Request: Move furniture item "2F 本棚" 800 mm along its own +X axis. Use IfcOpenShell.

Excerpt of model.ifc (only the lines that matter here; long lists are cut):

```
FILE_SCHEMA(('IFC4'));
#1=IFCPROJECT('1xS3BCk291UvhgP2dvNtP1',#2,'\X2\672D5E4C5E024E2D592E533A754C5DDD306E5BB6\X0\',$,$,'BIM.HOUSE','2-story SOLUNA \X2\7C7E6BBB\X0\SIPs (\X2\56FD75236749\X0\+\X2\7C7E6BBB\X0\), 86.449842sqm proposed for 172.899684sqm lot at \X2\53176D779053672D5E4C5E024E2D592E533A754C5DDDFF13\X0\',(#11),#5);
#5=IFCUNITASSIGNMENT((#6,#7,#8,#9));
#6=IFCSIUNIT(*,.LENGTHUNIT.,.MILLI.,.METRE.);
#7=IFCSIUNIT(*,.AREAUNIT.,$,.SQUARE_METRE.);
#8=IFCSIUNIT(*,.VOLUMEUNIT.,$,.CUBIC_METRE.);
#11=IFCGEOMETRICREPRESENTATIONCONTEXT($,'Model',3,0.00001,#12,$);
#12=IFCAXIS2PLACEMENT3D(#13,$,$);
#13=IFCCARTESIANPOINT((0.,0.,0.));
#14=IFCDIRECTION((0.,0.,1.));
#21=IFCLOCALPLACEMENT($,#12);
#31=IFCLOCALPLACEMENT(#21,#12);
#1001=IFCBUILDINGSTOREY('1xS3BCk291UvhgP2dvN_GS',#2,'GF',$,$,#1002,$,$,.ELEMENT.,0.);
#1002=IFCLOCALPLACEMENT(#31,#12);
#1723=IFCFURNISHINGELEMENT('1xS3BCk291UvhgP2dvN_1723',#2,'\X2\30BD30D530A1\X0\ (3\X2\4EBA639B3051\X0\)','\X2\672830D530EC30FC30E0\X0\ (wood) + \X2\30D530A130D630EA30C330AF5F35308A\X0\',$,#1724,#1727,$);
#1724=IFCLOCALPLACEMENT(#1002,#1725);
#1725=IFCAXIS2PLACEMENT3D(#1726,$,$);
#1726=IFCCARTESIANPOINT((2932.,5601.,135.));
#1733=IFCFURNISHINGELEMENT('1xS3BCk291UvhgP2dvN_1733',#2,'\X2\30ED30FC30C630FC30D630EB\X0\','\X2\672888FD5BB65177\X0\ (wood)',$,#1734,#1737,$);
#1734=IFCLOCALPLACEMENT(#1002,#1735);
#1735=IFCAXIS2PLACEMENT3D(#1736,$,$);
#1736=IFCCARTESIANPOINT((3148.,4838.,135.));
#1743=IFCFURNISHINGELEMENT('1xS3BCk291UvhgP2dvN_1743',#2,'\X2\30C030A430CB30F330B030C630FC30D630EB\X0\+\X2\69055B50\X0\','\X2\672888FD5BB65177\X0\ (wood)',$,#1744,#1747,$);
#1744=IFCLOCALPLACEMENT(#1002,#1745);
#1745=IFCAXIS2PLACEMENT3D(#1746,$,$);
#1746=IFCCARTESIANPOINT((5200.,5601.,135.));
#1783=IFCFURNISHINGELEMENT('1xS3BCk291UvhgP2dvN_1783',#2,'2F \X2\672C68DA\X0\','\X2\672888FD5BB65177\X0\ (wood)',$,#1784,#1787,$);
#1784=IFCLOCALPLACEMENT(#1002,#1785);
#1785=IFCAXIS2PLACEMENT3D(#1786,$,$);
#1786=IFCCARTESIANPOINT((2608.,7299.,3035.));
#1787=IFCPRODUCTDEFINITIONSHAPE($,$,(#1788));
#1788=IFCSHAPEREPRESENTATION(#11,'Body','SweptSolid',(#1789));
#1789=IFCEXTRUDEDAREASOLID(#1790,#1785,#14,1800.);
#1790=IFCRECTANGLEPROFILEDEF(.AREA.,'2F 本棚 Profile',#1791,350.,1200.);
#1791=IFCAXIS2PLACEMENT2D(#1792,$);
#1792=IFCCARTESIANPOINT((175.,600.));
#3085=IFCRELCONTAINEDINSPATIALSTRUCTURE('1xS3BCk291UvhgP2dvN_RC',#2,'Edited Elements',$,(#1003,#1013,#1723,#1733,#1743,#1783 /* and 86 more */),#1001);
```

```python
import ifcopenshell
import ifcopenshell.api.geometry
import ifcopenshell.util.placement
import ifcopenshell.util.unit

model = ifcopenshell.open("model.ifc")
unit_scale = ifcopenshell.util.unit.calculate_unit_scale(model)

item = model.by_guid("1xS3BCk291UvhgP2dvN_1783")
matrix = ifcopenshell.util.placement.get_local_placement(item.ObjectPlacement)
matrix[:3, 3] += matrix[:3, 0] * 0.8 / unit_scale
ifcopenshell.api.geometry.edit_object_placement(model, product=item, matrix=matrix, is_si=False)

print(ifcopenshell.util.placement.get_local_placement(item.ObjectPlacement).round(3) + 0.0)

model.write("model_rev.ifc")
```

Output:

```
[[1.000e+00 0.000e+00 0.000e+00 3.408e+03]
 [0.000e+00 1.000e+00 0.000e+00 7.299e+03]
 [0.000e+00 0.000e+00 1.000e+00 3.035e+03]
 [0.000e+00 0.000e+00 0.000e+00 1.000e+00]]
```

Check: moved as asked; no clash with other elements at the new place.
